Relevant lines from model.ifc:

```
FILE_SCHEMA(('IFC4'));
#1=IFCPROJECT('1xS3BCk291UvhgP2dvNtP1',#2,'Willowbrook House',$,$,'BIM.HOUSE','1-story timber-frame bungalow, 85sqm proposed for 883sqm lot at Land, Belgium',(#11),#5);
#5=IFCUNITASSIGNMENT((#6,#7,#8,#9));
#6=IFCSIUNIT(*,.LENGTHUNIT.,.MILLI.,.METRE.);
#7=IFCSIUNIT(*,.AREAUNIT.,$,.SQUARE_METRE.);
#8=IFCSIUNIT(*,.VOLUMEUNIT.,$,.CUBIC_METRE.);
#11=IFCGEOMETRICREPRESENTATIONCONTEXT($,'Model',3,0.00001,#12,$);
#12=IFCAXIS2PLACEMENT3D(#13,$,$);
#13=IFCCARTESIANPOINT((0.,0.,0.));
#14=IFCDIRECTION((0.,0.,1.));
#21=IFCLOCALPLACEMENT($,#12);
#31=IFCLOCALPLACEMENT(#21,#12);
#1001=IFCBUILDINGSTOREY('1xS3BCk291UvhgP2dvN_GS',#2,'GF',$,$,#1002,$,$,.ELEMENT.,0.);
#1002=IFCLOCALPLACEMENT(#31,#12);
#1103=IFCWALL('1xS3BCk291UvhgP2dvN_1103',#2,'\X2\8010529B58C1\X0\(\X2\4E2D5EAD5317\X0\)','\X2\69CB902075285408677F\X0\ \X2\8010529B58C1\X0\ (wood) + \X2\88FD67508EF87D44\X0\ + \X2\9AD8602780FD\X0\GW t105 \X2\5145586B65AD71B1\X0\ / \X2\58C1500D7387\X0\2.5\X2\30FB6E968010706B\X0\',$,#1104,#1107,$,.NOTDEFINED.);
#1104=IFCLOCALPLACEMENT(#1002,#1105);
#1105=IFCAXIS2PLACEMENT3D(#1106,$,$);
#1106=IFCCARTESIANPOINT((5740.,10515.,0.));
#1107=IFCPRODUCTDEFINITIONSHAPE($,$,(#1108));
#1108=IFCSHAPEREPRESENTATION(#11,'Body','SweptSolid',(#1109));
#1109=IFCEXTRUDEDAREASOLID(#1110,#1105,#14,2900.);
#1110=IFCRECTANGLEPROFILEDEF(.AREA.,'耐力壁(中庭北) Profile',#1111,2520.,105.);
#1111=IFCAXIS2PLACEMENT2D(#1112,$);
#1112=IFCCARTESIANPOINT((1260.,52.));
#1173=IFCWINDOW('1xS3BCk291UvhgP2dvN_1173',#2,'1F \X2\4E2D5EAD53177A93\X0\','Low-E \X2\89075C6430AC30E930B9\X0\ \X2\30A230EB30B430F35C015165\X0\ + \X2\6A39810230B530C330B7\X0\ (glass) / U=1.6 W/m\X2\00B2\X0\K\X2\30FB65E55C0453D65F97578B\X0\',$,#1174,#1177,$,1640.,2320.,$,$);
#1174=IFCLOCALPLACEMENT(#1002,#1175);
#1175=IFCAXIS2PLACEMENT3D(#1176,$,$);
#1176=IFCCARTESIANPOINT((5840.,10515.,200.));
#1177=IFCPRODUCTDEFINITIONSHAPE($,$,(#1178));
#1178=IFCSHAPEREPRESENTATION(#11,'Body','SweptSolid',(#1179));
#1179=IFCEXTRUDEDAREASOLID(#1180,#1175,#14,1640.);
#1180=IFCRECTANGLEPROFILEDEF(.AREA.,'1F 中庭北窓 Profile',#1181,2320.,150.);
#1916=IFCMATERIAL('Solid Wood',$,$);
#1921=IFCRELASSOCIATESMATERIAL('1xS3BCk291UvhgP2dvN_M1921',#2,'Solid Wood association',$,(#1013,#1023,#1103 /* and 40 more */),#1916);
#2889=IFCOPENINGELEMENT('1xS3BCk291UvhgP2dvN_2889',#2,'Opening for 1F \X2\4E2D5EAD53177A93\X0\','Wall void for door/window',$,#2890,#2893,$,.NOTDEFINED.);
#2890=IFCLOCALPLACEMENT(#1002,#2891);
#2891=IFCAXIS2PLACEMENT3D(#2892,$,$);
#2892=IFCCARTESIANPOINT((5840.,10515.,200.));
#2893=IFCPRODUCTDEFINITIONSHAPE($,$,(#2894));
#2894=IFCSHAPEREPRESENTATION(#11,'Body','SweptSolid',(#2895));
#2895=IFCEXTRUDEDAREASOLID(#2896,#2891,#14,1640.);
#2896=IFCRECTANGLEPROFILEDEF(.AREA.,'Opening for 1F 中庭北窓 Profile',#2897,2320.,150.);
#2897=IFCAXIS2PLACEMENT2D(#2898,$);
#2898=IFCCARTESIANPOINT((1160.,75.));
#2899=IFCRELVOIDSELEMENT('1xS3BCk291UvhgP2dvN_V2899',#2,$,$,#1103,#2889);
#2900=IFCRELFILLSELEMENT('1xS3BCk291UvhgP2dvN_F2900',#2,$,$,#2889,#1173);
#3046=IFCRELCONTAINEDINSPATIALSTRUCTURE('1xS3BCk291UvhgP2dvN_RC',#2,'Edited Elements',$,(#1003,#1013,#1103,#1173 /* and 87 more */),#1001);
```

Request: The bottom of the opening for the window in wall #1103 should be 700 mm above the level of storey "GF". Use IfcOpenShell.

```python
import numpy as np
import ifcopenshell
import ifcopenshell.api.geometry
import ifcopenshell.geom
import ifcopenshell.util.element
import ifcopenshell.util.placement
import ifcopenshell.util.shape
import ifcopenshell.util.unit

model = ifcopenshell.open("model.ifc")
unit_scale = ifcopenshell.util.unit.calculate_unit_scale(model)

window = model.by_guid("1xS3BCk291UvhgP2dvN_1173")
opening = window.FillsVoids[0].RelatingOpeningElement
storey = ifcopenshell.util.element.get_container(window, ifc_class="IfcBuildingStorey")
level = ifcopenshell.util.placement.get_local_placement(storey.ObjectPlacement)[2, 3]

# The opening's origin need not be at the sill, so measure its lowest point.
shape = ifcopenshell.geom.create_shape(ifcopenshell.geom.settings(), opening)
bottom = ifcopenshell.util.shape.get_shape_bottom_elevation(shape, shape.geometry) / unit_scale
dz = level + 0.7 / unit_scale - bottom

shift = np.array([0.0, 0.0, dz])
# The window is not placed relative to its opening, so move both.
for product in (opening, window):
    matrix = ifcopenshell.util.placement.get_local_placement(product.ObjectPlacement)
    matrix[:3, 3] += shift
    ifcopenshell.api.geometry.edit_object_placement(model, product=product, matrix=matrix, is_si=False)

print(f"moved by {dz * unit_scale:+.3f} m")

model.write("model_v2.ifc")
```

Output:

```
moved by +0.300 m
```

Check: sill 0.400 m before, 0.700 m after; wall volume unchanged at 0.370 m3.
